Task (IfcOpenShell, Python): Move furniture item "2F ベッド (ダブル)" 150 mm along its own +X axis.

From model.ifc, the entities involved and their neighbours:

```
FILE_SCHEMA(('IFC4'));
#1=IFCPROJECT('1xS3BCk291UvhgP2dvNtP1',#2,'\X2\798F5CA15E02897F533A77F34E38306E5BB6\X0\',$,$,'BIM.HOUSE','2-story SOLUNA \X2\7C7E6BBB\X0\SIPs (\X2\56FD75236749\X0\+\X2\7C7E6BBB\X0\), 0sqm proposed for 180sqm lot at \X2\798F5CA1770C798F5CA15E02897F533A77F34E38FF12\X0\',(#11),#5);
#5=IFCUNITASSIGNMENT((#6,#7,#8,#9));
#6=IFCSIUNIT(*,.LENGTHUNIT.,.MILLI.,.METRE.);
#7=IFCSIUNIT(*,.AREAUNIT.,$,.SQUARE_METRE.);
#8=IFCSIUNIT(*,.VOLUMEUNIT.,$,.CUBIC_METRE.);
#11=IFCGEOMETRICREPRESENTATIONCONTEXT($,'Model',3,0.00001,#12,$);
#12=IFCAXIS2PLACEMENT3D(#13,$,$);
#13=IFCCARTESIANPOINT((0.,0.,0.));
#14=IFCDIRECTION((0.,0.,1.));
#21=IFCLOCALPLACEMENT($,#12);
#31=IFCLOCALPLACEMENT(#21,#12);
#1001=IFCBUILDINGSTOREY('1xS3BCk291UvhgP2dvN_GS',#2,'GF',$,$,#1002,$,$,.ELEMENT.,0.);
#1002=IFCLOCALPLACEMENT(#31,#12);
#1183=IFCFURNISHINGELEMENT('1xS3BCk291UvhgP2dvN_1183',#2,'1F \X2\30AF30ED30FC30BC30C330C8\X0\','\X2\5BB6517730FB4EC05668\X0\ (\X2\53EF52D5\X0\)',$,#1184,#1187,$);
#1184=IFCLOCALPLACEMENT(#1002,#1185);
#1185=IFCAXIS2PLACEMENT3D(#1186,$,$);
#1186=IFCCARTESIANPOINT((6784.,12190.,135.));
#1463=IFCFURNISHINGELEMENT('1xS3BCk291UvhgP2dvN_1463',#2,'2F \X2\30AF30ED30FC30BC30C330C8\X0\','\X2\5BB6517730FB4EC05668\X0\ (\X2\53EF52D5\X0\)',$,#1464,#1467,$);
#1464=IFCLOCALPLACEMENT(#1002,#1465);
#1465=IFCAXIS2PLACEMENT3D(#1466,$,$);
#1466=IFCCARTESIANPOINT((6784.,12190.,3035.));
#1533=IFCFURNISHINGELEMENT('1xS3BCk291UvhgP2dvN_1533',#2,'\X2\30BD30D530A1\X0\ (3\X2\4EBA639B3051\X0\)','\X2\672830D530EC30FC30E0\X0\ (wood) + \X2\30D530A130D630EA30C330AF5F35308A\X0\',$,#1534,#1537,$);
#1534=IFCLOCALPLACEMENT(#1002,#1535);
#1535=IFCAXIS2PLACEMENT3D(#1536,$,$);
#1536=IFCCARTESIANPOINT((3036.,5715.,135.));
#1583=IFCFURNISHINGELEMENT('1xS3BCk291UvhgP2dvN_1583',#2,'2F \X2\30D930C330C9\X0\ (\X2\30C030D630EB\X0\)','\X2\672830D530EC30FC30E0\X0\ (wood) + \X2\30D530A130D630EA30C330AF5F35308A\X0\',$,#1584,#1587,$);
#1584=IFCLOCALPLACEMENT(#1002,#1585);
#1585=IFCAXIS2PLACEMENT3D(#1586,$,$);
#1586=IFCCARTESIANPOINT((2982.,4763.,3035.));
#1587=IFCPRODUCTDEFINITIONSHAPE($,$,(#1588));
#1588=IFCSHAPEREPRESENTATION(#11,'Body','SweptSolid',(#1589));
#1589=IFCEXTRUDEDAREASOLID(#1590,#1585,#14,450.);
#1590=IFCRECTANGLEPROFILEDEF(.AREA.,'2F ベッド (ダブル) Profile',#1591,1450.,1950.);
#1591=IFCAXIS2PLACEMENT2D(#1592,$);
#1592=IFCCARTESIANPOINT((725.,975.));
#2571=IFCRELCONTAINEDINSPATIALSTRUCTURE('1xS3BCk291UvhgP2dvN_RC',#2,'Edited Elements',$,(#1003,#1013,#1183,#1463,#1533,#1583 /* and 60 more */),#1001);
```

```python
import ifcopenshell
import ifcopenshell.api.geometry
import ifcopenshell.util.placement
import ifcopenshell.util.unit

model = ifcopenshell.open("model.ifc")
unit_scale = ifcopenshell.util.unit.calculate_unit_scale(model)

item = model.by_id(1583)
matrix = ifcopenshell.util.placement.get_local_placement(item.ObjectPlacement)
matrix[:3, 3] += matrix[:3, 0] * 0.15 / unit_scale
ifcopenshell.api.geometry.edit_object_placement(model, product=item, matrix=matrix, is_si=False)

print(ifcopenshell.util.placement.get_local_placement(item.ObjectPlacement).round(3) + 0.0)

model.write("model_updated.ifc")
```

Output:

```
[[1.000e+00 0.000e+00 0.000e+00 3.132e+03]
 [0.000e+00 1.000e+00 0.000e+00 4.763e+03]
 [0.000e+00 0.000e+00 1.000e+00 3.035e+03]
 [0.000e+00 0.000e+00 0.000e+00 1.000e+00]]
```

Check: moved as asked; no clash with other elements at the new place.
